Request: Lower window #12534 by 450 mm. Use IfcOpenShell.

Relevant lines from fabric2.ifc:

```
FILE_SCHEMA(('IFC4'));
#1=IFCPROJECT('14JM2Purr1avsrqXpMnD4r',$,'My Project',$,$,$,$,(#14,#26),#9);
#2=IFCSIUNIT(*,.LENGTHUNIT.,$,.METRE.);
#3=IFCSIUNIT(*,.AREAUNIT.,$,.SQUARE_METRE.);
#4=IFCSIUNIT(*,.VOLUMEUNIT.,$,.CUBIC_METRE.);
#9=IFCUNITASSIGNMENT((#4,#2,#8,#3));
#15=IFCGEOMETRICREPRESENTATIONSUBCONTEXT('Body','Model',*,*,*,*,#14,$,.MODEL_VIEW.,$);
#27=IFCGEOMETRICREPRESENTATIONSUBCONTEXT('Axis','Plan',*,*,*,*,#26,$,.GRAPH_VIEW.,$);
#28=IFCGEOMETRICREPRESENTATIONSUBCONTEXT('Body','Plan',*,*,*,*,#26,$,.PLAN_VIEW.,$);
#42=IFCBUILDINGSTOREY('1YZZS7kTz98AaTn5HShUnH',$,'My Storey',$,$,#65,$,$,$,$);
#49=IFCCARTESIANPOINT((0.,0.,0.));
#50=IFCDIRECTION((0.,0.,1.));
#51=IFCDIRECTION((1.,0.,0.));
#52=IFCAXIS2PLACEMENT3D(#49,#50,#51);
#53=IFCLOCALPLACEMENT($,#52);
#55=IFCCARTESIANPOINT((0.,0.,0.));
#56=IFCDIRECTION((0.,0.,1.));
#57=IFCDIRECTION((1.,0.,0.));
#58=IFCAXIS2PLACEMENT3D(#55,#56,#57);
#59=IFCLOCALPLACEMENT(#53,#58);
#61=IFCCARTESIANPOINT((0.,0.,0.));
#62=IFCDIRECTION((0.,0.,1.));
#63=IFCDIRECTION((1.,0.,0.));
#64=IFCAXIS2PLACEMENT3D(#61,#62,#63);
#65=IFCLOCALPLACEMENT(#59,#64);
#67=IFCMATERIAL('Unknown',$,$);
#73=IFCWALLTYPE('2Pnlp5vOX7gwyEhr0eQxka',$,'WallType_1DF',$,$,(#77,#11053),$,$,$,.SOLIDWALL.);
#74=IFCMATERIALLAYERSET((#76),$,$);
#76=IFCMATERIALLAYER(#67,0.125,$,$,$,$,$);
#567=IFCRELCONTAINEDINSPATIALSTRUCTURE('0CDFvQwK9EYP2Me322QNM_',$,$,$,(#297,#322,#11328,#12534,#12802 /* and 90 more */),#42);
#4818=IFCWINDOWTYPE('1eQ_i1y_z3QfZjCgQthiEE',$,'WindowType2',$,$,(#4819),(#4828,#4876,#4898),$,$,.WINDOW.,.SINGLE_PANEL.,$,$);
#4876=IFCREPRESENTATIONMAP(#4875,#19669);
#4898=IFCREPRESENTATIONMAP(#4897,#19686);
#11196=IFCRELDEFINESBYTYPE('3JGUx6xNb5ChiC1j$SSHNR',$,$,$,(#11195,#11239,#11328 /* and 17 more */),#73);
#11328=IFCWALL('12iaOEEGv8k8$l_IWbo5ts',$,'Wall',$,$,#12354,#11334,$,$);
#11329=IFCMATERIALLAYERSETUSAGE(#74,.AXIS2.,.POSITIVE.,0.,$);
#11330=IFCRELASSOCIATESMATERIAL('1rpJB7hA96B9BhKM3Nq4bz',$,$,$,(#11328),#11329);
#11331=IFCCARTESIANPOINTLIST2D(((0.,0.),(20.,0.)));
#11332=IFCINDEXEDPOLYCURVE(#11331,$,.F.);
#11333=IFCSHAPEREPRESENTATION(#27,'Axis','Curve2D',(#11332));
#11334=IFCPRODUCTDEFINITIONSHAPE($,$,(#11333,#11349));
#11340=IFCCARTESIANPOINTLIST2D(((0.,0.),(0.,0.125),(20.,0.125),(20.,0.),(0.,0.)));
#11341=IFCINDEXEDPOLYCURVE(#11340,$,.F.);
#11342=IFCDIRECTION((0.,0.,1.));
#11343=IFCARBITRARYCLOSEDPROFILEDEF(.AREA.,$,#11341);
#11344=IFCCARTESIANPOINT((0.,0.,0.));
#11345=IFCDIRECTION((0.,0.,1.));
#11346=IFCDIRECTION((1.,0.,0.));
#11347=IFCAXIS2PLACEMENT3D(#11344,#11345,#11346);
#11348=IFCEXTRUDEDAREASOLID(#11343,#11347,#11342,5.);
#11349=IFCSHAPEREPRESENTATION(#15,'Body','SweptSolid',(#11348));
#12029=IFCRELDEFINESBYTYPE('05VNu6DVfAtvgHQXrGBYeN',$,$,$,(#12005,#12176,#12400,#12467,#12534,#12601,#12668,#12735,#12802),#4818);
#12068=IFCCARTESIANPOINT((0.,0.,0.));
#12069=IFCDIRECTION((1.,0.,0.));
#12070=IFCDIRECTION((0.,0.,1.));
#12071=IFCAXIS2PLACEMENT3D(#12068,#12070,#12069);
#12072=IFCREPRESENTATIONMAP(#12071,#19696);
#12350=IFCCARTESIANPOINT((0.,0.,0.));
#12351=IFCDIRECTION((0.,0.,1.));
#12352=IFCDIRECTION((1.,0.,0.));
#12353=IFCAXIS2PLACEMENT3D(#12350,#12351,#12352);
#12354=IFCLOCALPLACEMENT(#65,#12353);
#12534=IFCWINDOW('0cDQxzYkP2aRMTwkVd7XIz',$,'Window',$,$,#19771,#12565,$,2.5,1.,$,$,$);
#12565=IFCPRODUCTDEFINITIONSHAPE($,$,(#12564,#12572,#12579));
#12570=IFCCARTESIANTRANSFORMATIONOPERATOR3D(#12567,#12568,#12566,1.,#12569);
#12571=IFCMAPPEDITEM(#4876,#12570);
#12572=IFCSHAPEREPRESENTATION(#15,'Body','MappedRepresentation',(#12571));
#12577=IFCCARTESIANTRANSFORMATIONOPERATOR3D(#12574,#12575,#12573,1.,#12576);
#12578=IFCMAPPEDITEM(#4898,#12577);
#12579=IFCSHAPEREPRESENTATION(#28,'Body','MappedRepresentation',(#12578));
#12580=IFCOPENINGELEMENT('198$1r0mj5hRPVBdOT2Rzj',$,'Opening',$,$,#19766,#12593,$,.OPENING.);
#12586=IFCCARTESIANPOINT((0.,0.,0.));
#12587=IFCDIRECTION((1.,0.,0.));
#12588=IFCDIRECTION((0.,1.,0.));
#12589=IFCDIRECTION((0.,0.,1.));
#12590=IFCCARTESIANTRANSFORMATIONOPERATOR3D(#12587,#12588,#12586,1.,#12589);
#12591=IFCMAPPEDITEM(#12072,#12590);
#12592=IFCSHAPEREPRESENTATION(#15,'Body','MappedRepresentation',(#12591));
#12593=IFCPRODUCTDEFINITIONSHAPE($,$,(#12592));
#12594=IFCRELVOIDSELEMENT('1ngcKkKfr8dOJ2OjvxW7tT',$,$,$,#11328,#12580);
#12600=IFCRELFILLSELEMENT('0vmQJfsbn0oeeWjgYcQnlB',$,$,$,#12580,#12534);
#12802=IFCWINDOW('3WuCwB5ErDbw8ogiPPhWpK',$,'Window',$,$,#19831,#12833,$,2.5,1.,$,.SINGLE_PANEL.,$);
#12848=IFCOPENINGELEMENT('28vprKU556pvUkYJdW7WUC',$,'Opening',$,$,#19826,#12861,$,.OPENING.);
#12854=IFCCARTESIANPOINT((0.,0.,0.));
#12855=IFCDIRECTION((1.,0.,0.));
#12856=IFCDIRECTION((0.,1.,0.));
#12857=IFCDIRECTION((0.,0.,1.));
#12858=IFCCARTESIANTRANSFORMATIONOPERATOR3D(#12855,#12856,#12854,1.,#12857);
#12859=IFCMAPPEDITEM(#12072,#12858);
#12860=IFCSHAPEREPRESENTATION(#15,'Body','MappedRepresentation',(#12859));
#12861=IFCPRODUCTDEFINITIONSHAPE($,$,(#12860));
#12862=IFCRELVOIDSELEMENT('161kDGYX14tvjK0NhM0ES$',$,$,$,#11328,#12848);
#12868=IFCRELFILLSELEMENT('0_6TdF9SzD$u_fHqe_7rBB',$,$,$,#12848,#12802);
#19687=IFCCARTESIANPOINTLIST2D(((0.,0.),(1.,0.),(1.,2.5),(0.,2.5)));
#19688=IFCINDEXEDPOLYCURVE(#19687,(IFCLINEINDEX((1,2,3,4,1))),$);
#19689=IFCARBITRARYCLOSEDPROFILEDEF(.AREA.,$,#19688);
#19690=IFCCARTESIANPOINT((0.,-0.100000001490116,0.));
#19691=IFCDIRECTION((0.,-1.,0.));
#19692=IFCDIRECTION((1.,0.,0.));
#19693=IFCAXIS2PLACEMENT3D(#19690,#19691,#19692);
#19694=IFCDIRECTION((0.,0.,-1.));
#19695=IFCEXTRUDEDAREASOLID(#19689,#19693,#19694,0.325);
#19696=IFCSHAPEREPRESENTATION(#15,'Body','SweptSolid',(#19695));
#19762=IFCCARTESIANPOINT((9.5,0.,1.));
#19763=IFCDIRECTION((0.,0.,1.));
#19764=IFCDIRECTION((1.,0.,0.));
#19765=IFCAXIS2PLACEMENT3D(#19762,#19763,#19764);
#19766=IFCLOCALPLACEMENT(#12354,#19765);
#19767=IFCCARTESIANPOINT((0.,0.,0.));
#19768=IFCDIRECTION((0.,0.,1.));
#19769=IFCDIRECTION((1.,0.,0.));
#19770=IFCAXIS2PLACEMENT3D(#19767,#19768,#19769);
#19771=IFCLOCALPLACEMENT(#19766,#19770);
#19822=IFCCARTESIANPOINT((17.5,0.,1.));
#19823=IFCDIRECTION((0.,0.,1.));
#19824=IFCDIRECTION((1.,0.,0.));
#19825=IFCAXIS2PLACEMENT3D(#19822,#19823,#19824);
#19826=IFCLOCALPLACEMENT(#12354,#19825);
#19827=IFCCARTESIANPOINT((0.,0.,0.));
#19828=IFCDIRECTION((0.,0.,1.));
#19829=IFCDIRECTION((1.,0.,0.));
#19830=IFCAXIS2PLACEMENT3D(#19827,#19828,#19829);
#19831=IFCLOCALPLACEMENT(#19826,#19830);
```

```python
import numpy as np
import ifcopenshell
import ifcopenshell.api.geometry
import ifcopenshell.util.placement
import ifcopenshell.util.unit

model = ifcopenshell.open("fabric2.ifc")
unit_scale = ifcopenshell.util.unit.calculate_unit_scale(model)

window = model.by_guid("0cDQxzYkP2aRMTwkVd7XIz")
opening = window.FillsVoids[0].RelatingOpeningElement
dz = -0.45

shift = np.array([0.0, 0.0, dz])
# The window is placed relative to its opening, so it follows when the opening moves.
matrix = ifcopenshell.util.placement.get_local_placement(opening.ObjectPlacement)
matrix[:3, 3] += shift
ifcopenshell.api.geometry.edit_object_placement(
    model, product=opening, matrix=matrix, is_si=False, should_transform_children=True
)

print(f"moved by {dz * unit_scale:+.3f} m")

model.write("fabric2_rev.ifc")
```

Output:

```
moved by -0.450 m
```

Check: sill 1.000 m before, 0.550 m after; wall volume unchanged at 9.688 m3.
